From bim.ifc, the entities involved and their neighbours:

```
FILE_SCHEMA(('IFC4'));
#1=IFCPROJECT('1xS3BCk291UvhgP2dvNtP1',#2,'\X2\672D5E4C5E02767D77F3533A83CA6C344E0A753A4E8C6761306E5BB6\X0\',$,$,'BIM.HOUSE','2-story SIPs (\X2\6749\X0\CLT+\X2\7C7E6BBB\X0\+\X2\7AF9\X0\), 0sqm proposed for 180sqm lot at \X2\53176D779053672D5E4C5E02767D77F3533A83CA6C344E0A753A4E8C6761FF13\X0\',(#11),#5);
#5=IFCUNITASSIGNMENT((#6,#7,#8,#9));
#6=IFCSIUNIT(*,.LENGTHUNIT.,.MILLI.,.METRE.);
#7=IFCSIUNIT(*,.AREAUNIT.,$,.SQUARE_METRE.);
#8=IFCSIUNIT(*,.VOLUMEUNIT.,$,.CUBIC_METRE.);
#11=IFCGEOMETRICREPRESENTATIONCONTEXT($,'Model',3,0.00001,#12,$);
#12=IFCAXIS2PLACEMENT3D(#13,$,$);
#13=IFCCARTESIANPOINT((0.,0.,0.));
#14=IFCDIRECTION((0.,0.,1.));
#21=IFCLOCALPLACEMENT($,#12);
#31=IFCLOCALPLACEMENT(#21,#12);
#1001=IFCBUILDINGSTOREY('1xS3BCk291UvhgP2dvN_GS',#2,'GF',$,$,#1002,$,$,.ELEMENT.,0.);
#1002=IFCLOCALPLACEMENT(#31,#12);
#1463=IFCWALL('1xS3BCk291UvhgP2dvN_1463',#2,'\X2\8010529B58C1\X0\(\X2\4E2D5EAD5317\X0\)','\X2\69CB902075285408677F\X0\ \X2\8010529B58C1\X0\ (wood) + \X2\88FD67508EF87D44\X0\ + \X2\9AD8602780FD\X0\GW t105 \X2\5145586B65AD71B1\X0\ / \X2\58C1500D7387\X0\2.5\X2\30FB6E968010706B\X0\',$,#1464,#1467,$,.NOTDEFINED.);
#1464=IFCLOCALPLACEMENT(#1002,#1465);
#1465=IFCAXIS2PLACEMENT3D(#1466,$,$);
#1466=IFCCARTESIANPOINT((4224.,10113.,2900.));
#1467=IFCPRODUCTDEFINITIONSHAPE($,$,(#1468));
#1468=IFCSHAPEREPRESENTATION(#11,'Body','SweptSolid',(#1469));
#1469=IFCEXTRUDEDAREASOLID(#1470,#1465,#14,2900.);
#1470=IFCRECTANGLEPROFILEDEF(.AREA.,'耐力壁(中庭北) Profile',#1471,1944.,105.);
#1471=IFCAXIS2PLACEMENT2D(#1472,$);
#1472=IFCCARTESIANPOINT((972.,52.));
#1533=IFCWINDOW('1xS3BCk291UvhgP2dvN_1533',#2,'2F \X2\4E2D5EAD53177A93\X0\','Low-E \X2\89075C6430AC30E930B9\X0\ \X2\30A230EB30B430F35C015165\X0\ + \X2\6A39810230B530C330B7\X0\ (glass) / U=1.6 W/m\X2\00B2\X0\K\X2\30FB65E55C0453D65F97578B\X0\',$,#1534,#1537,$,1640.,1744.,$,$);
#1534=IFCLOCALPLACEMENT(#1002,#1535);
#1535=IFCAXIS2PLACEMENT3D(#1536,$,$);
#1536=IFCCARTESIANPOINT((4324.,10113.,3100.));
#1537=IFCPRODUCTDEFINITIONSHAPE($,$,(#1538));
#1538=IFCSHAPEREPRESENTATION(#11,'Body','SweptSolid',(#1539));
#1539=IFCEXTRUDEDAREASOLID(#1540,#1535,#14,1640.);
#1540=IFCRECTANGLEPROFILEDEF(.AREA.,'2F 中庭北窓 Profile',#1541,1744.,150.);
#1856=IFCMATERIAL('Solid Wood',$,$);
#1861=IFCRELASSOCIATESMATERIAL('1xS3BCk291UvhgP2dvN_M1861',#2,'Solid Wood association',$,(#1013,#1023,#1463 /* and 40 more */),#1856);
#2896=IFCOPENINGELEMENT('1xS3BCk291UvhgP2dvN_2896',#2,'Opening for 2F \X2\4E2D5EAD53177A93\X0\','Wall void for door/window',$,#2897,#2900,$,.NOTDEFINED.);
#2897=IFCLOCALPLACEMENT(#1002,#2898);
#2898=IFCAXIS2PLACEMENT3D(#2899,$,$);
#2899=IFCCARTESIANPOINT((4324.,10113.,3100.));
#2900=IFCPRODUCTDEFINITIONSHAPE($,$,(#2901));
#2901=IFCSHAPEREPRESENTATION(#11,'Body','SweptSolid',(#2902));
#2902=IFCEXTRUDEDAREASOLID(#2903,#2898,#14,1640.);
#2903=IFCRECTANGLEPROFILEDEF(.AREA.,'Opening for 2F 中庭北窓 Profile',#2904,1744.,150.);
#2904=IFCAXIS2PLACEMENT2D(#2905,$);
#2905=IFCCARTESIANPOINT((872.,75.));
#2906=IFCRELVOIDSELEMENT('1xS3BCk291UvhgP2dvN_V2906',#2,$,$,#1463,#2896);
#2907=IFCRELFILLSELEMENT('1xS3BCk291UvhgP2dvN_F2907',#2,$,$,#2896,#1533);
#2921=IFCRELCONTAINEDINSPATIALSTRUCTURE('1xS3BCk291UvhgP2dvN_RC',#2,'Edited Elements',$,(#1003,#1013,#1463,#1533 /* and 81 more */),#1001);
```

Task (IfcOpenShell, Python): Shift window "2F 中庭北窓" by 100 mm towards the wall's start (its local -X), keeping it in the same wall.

```python
import ifcopenshell
import ifcopenshell.api.geometry
import ifcopenshell.util.placement

model = ifcopenshell.open("bim.ifc")

window = model.by_guid("1xS3BCk291UvhgP2dvN_1533")
opening = window.FillsVoids[0].RelatingOpeningElement
wall = opening.VoidsElements[0].RelatingBuildingElement

wall_matrix = ifcopenshell.util.placement.get_local_placement(wall.ObjectPlacement)
shift = wall_matrix[:3, 0] * -100.0
before = ifcopenshell.util.placement.get_local_placement(window.ObjectPlacement)[:3, 3].copy()

# The window is not placed relative to its opening, so move both.
for product in (opening, window):
    matrix = ifcopenshell.util.placement.get_local_placement(product.ObjectPlacement)
    matrix[:3, 3] += shift
    ifcopenshell.api.geometry.edit_object_placement(model, product=product, matrix=matrix, is_si=False)

after = ifcopenshell.util.placement.get_local_placement(window.ObjectPlacement)[:3, 3]
print("window moved by", (after - before).round(3) + 0.0)

model.write("bim-out.ifc")
```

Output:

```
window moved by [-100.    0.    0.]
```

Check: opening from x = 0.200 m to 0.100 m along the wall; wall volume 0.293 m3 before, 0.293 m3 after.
